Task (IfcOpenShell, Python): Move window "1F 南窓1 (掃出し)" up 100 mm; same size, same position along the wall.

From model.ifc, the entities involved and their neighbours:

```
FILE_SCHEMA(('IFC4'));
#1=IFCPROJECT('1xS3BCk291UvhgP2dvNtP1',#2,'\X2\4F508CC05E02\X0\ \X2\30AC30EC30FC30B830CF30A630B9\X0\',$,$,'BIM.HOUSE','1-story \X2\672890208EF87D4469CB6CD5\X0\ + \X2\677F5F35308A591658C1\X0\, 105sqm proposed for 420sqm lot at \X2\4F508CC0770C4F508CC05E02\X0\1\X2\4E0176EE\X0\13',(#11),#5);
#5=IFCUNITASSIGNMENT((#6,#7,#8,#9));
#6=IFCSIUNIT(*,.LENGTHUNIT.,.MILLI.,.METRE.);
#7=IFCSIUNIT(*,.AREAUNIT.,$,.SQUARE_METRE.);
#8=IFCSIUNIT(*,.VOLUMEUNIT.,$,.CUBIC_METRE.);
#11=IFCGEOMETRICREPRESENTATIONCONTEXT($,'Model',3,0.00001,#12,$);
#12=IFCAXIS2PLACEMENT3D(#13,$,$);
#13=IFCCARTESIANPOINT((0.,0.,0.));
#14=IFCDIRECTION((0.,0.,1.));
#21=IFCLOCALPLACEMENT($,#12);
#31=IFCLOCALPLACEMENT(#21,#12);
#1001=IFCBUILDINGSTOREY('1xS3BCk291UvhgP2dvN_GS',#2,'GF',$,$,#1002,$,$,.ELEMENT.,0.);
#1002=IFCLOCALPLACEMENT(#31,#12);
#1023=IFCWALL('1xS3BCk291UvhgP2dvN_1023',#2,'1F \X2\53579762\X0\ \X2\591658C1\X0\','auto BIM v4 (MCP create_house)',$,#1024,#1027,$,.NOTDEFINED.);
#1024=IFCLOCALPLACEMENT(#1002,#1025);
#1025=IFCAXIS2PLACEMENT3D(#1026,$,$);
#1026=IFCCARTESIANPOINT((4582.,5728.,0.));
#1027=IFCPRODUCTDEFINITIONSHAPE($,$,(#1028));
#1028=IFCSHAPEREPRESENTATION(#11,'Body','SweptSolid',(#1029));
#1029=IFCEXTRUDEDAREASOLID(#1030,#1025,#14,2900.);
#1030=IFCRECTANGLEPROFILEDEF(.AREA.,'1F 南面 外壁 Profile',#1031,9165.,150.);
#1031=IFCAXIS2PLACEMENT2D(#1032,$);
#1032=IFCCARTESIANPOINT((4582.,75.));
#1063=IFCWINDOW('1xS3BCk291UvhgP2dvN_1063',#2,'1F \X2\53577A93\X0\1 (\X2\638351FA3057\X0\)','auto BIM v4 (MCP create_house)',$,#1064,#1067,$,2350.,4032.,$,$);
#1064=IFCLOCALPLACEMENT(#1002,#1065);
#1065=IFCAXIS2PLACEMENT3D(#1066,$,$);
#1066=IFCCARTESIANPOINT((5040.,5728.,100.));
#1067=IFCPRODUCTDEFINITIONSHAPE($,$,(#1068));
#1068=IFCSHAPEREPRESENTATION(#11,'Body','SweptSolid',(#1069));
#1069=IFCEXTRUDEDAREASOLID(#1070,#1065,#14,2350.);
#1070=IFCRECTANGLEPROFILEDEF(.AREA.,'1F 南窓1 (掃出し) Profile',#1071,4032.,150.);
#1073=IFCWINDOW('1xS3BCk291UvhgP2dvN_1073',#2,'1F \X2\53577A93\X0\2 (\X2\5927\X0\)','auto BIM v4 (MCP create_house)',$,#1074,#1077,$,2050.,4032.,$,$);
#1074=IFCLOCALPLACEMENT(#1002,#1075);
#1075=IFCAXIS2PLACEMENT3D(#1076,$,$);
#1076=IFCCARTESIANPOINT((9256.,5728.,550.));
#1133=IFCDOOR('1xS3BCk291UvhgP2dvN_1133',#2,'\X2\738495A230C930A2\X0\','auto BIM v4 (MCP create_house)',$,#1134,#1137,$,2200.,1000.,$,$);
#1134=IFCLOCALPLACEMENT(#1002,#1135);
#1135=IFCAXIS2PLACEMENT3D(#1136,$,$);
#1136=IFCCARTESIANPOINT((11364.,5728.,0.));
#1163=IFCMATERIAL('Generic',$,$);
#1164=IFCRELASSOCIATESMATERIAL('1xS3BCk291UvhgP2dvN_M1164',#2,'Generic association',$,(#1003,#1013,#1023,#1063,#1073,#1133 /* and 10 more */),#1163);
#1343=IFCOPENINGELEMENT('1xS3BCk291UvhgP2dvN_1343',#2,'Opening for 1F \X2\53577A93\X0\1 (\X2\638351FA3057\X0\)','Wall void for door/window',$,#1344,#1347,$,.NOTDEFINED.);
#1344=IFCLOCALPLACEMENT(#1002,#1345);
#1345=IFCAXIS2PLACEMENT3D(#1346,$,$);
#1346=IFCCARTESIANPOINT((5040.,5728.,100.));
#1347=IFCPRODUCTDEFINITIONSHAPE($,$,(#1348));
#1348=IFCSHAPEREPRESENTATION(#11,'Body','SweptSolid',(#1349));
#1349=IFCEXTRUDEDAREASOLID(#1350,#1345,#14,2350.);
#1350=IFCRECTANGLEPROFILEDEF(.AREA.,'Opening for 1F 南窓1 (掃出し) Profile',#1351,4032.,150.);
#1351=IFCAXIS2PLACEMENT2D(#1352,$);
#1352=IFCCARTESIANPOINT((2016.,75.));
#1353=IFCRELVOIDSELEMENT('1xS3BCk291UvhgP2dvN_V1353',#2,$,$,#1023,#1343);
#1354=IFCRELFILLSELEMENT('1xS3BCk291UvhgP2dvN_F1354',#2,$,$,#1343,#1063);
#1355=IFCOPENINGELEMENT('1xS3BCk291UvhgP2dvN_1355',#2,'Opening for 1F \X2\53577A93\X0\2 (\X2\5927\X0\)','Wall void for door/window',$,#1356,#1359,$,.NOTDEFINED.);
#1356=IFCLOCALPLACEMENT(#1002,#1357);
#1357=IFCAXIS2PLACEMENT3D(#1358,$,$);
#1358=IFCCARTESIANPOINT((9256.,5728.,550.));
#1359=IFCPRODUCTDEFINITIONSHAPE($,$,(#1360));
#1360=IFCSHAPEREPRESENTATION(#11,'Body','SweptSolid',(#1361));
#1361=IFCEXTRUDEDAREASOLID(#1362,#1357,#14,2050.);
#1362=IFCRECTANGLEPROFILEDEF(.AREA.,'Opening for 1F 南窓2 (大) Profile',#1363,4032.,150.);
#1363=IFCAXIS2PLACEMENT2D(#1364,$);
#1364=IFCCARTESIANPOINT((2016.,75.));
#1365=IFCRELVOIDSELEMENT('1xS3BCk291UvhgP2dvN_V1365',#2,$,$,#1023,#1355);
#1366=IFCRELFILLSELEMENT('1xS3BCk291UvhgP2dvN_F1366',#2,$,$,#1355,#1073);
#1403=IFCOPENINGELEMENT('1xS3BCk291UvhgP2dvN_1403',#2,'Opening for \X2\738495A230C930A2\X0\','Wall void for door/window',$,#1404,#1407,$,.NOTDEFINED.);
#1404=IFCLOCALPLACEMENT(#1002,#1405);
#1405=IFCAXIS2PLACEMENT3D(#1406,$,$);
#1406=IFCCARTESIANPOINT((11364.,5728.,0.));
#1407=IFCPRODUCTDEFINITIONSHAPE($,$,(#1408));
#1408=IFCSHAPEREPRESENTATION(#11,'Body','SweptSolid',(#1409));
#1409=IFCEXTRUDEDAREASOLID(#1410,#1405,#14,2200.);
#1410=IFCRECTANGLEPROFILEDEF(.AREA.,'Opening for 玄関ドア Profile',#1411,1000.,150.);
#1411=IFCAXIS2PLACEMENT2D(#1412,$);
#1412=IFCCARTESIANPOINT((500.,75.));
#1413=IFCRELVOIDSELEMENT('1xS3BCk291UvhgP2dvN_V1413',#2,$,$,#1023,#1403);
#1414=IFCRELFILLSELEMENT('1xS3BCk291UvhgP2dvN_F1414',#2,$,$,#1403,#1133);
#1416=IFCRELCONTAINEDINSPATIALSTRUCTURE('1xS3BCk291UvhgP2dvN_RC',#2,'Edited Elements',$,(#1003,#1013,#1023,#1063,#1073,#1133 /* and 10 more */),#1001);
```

```python
import numpy as np
import ifcopenshell
import ifcopenshell.api.geometry
import ifcopenshell.util.placement
import ifcopenshell.util.unit

model = ifcopenshell.open("model.ifc")
unit_scale = ifcopenshell.util.unit.calculate_unit_scale(model)

window = model.by_guid("1xS3BCk291UvhgP2dvN_1063")
opening = window.FillsVoids[0].RelatingOpeningElement
dz = 0.1 / unit_scale

shift = np.array([0.0, 0.0, dz])
# The window is not placed relative to its opening, so move both.
for product in (opening, window):
    matrix = ifcopenshell.util.placement.get_local_placement(product.ObjectPlacement)
    matrix[:3, 3] += shift
    ifcopenshell.api.geometry.edit_object_placement(model, product=product, matrix=matrix, is_si=False)

print(f"moved by {dz * unit_scale:+.3f} m")

model.write("model-out.ifc")
```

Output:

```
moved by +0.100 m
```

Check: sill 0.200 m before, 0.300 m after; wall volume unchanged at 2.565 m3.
